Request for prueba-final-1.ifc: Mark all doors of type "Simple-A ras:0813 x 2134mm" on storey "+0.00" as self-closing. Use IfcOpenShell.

First a look at what the model holds.

```python
import ifcopenshell
import ifcopenshell.util.element

model = ifcopenshell.open("prueba-final-1.ifc")
print(model.schema)
storey = next(s for s in model.by_type("IfcBuildingStorey") if s.Name == "+0.00")
doors = [e for e in ifcopenshell.util.element.get_decomposition(storey) if e.is_a("IfcDoor")]
seen = {}
for e in doors:
    element_type = ifcopenshell.util.element.get_type(e)
    key = (element_type.Name if element_type != e and element_type else None, ifcopenshell.util.element.get_pset(e, "Pset_DoorCommon", "SelfClosing"))
    seen[key] = seen.get(key, 0) + 1
for (name, value), count in sorted(seen.items(), key=str):
    print(count, "x", name, "|", value)
```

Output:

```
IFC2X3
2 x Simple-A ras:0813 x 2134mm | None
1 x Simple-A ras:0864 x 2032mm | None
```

```python
import ifcopenshell
import ifcopenshell.api.pset
import ifcopenshell.util.element

model = ifcopenshell.open("prueba-final-1.ifc")

storey = next(s for s in model.by_type("IfcBuildingStorey") if s.Name == "+0.00")
doors = [e for e in ifcopenshell.util.element.get_decomposition(storey) if e.is_a("IfcDoor")]

count = 0
for e in doors:
    element_type = ifcopenshell.util.element.get_type(e)
    if element_type in (None, e) or element_type.Name != "Simple-A ras:0813 x 2134mm":
        continue
    # add_pset returns the element's existing set when there is one.
    pset = ifcopenshell.api.pset.add_pset(model, product=e, name="Pset_DoorCommon")
    ifcopenshell.api.pset.edit_pset(model, pset=pset, properties={"SelfClosing": True})
    count += 1

print(count, "doors updated")

model.write("prueba-final-1-out.ifc")
```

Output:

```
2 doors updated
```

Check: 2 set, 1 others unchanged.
